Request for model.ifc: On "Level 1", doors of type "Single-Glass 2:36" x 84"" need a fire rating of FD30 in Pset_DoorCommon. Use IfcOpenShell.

First a look at what the model holds.

```python
import ifcopenshell
import ifcopenshell.util.element

model = ifcopenshell.open("model.ifc")
print(model.schema)
storey = next(s for s in model.by_type("IfcBuildingStorey") if s.Name == "Level 1")
doors = [e for e in ifcopenshell.util.element.get_decomposition(storey) if e.is_a("IfcDoor")]
seen = {}
for e in doors:
    element_type = ifcopenshell.util.element.get_type(e)
    key = (element_type.Name if element_type != e and element_type else None, ifcopenshell.util.element.get_pset(e, "Pset_DoorCommon", "FireRating"))
    seen[key] = seen.get(key, 0) + 1
for (name, value), count in sorted(seen.items(), key=str):
    print(count, "x", name, "|", value)
```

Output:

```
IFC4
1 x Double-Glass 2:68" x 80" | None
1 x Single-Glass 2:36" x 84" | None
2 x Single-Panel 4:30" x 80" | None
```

```python
import ifcopenshell
import ifcopenshell.api.pset
import ifcopenshell.util.element

model = ifcopenshell.open("model.ifc")

storey = next(s for s in model.by_type("IfcBuildingStorey") if s.Name == "Level 1")
doors = [e for e in ifcopenshell.util.element.get_decomposition(storey) if e.is_a("IfcDoor")]

count = 0
for e in doors:
    element_type = ifcopenshell.util.element.get_type(e)
    if element_type in (None, e) or element_type.Name != 'Single-Glass 2:36" x 84"':
        continue
    # add_pset returns the element's existing set when there is one.
    pset = ifcopenshell.api.pset.add_pset(model, product=e, name="Pset_DoorCommon")
    ifcopenshell.api.pset.edit_pset(model, pset=pset, properties={"FireRating": "FD30"})
    count += 1

print(count, "doors updated")

model.write("model-out.ifc")
```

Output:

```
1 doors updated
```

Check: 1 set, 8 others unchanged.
